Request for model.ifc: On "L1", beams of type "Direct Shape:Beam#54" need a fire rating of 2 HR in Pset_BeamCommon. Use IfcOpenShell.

First a look at what the model holds.

```python
import ifcopenshell
import ifcopenshell.util.element

model = ifcopenshell.open("model.ifc")
print(model.schema)
storey = next(s for s in model.by_type("IfcBuildingStorey") if s.Name == "L1")
beams = [e for e in ifcopenshell.util.element.get_decomposition(storey) if e.is_a("IfcBeam")]
seen = {}
for e in beams:
    element_type = ifcopenshell.util.element.get_type(e)
    key = (element_type.Name if element_type != e and element_type else None, ifcopenshell.util.element.get_pset(e, "Pset_BeamCommon", "FireRating"))
    seen[key] = seen.get(key, 0) + 1
for (name, value), count in sorted(seen.items(), key=str):
    print(count, "x", name, "|", value)
```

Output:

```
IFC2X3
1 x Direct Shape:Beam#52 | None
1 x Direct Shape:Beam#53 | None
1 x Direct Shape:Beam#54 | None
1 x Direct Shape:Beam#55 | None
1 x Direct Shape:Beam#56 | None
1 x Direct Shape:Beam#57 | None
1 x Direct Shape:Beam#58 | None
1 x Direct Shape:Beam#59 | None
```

```python
import ifcopenshell
import ifcopenshell.api.pset
import ifcopenshell.util.element

model = ifcopenshell.open("model.ifc")

storey = next(s for s in model.by_type("IfcBuildingStorey") if s.Name == "L1")
beams = [e for e in ifcopenshell.util.element.get_decomposition(storey) if e.is_a("IfcBeam")]

count = 0
for e in beams:
    element_type = ifcopenshell.util.element.get_type(e)
    if element_type in (None, e) or element_type.Name != "Direct Shape:Beam#54":
        continue
    # add_pset returns the element's existing set when there is one.
    pset = ifcopenshell.api.pset.add_pset(model, product=e, name="Pset_BeamCommon")
    ifcopenshell.api.pset.edit_pset(model, pset=pset, properties={"FireRating": "2 HR"})
    count += 1

print(count, "beams updated")

model.write("model-out.ifc")
```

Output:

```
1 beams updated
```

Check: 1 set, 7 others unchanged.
